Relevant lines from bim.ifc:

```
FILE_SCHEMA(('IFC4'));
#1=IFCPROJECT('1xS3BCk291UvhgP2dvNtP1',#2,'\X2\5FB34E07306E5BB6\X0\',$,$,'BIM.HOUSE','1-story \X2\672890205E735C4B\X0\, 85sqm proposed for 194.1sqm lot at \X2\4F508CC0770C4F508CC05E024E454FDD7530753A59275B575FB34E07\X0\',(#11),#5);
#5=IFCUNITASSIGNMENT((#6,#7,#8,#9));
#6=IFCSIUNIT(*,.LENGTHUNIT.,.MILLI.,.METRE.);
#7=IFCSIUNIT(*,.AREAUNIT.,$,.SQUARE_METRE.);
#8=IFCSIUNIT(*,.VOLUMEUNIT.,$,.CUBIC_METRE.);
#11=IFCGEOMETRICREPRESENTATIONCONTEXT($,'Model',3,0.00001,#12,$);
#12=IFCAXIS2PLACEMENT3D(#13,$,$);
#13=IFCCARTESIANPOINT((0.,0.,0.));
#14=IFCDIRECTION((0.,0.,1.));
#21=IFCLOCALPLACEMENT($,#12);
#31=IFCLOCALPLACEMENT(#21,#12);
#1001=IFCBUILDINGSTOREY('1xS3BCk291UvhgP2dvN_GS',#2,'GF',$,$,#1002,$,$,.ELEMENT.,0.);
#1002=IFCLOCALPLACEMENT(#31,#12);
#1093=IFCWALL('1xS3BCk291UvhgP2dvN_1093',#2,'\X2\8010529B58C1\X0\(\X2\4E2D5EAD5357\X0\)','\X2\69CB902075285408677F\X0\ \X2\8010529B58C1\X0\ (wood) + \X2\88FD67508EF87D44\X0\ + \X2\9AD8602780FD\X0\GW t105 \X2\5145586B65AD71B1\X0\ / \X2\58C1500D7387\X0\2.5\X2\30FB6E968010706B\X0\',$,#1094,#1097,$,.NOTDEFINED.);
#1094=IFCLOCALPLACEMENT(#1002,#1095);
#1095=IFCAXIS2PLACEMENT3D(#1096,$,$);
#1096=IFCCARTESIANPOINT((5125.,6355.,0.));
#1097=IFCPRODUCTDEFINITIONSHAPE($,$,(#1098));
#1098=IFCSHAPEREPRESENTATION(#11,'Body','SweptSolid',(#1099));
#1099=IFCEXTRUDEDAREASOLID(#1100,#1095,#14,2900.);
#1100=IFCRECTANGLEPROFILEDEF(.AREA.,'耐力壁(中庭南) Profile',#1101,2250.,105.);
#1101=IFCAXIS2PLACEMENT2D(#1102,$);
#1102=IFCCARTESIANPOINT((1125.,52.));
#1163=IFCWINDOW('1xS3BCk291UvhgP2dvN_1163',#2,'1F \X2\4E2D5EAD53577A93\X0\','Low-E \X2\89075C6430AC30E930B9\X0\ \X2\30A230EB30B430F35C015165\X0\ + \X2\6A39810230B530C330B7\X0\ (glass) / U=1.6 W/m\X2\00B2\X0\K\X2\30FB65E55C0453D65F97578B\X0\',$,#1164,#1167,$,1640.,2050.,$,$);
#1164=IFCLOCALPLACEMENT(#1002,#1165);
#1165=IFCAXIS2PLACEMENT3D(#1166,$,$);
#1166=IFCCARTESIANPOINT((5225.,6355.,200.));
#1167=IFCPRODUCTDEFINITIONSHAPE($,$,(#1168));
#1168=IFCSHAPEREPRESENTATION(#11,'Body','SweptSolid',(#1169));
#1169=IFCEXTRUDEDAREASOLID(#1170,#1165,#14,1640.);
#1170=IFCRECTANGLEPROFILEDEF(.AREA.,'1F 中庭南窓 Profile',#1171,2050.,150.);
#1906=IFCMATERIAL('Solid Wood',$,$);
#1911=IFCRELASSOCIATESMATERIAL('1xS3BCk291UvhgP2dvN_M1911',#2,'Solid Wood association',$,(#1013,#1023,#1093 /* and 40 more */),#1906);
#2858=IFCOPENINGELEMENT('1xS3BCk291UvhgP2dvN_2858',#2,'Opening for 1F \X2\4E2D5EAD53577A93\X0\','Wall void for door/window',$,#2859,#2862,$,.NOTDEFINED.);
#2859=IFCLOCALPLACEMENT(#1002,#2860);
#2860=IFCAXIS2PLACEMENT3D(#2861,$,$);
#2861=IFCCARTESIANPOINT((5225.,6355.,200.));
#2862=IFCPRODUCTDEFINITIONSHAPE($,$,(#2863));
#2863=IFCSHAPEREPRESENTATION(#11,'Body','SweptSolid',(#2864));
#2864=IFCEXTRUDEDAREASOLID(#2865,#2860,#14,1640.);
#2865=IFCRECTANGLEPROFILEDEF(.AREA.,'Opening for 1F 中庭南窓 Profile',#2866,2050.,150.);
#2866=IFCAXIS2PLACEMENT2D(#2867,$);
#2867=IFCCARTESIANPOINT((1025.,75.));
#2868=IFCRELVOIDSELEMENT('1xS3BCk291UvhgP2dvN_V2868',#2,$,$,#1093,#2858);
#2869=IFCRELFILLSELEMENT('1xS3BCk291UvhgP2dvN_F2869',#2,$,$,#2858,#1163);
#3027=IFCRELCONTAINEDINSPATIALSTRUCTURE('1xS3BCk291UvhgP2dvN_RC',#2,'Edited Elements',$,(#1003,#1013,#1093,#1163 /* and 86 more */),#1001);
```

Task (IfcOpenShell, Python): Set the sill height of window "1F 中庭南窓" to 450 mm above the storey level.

```python
import numpy as np
import ifcopenshell
import ifcopenshell.api.geometry
import ifcopenshell.geom
import ifcopenshell.util.element
import ifcopenshell.util.placement
import ifcopenshell.util.shape
import ifcopenshell.util.unit

model = ifcopenshell.open("bim.ifc")
unit_scale = ifcopenshell.util.unit.calculate_unit_scale(model)

window = model.by_id(1163)
opening = window.FillsVoids[0].RelatingOpeningElement
storey = ifcopenshell.util.element.get_container(window, ifc_class="IfcBuildingStorey")
level = ifcopenshell.util.placement.get_local_placement(storey.ObjectPlacement)[2, 3]

# The opening's origin need not be at the sill, so measure its lowest point.
shape = ifcopenshell.geom.create_shape(ifcopenshell.geom.settings(), opening)
bottom = ifcopenshell.util.shape.get_shape_bottom_elevation(shape, shape.geometry) / unit_scale
dz = level + 0.45 / unit_scale - bottom

shift = np.array([0.0, 0.0, dz])
# The window is not placed relative to its opening, so move both.
for product in (opening, window):
    matrix = ifcopenshell.util.placement.get_local_placement(product.ObjectPlacement)
    matrix[:3, 3] += shift
    ifcopenshell.api.geometry.edit_object_placement(model, product=product, matrix=matrix, is_si=False)

print(f"moved by {dz * unit_scale:+.3f} m")

model.write("bim_edited.ifc")
```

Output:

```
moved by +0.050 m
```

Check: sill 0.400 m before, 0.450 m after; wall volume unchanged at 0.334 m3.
